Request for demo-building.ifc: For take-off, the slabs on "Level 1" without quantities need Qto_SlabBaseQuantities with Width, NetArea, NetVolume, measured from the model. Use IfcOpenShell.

First a look at what the model holds.

```python
import ifcopenshell
import ifcopenshell.util.element
import ifcopenshell.util.unit

model = ifcopenshell.open("demo-building.ifc")
print(model.schema)
for unit_type in ("LENGTHUNIT", "AREAUNIT", "VOLUMEUNIT"):
    print(unit_type, ifcopenshell.util.unit.calculate_unit_scale(model, unit_type))
storey = next(s for s in model.by_type("IfcBuildingStorey") if s.Name == "Level 1")
slabs = [e for e in ifcopenshell.util.element.get_decomposition(storey) if e.is_a("IfcSlab")]
for e in sorted(slabs, key=lambda e: e.id()):
    print(e.id(), e.is_a(), e.Name, list(ifcopenshell.util.element.get_psets(e, qtos_only=True)), sep=" | ")
```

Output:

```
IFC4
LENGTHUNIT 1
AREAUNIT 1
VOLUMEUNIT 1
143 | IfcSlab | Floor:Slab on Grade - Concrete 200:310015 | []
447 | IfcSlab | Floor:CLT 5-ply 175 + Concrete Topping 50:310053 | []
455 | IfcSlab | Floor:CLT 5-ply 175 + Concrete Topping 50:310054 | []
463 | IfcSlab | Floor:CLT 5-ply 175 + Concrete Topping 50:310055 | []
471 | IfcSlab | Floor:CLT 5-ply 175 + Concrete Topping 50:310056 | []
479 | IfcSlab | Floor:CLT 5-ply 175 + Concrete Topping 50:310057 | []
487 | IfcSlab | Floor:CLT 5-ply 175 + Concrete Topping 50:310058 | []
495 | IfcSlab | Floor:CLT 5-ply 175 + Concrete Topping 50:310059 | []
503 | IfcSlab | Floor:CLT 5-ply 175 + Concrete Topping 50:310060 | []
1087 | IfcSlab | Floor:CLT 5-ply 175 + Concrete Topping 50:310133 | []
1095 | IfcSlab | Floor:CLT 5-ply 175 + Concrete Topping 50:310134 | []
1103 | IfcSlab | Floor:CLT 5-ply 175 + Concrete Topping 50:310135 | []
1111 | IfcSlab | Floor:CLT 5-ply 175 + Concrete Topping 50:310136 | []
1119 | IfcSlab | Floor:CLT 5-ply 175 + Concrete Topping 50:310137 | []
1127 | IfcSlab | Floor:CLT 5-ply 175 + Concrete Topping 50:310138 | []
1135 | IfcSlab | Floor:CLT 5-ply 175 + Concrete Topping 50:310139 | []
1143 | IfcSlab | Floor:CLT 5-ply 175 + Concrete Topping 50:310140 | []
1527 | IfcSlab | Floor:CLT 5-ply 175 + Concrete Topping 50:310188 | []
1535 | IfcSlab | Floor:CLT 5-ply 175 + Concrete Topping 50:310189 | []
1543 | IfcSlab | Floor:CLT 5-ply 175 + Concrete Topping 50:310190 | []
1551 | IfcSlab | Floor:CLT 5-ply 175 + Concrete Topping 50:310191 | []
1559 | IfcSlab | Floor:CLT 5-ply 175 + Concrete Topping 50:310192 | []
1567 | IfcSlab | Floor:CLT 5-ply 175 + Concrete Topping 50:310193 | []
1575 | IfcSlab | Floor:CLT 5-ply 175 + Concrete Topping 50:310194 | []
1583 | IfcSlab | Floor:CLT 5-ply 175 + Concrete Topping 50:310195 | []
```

```python
import ifcopenshell
import ifcopenshell.api.pset
import ifcopenshell.geom
import ifcopenshell.util.element
import ifcopenshell.util.shape
import ifcopenshell.util.unit

model = ifcopenshell.open("demo-building.ifc")
unit_scale = ifcopenshell.util.unit.calculate_unit_scale(model)
area_scale = ifcopenshell.util.unit.calculate_unit_scale(model, "AREAUNIT")
volume_scale = ifcopenshell.util.unit.calculate_unit_scale(model, "VOLUMEUNIT")
settings = ifcopenshell.geom.settings()

storey = next(s for s in model.by_type("IfcBuildingStorey") if s.Name == "Level 1")
slabs = [e for e in ifcopenshell.util.element.get_decomposition(storey) if e.is_a("IfcSlab")]

for e in sorted(slabs, key=lambda e: e.id()):
    if ifcopenshell.util.element.get_psets(e, qtos_only=True, should_inherit=False):
        continue
    # Geometry comes back in metres, in the element's own axes.
    shape = ifcopenshell.geom.create_shape(settings, e)
    values = {
        "Width": ifcopenshell.util.shape.get_z(shape.geometry) / unit_scale,
        "NetArea": ifcopenshell.util.shape.get_footprint_area(shape.geometry) / area_scale,
        "NetVolume": ifcopenshell.util.shape.get_volume(shape.geometry) / volume_scale,
    }
    qto = ifcopenshell.api.pset.add_qto(model, product=e, name="Qto_SlabBaseQuantities")
    ifcopenshell.api.pset.edit_qto(model, qto=qto, properties=values)
    print(e.id(), {k: round(v, 3) for k, v in values.items()})

model.write("demo-building_updated.ifc")
```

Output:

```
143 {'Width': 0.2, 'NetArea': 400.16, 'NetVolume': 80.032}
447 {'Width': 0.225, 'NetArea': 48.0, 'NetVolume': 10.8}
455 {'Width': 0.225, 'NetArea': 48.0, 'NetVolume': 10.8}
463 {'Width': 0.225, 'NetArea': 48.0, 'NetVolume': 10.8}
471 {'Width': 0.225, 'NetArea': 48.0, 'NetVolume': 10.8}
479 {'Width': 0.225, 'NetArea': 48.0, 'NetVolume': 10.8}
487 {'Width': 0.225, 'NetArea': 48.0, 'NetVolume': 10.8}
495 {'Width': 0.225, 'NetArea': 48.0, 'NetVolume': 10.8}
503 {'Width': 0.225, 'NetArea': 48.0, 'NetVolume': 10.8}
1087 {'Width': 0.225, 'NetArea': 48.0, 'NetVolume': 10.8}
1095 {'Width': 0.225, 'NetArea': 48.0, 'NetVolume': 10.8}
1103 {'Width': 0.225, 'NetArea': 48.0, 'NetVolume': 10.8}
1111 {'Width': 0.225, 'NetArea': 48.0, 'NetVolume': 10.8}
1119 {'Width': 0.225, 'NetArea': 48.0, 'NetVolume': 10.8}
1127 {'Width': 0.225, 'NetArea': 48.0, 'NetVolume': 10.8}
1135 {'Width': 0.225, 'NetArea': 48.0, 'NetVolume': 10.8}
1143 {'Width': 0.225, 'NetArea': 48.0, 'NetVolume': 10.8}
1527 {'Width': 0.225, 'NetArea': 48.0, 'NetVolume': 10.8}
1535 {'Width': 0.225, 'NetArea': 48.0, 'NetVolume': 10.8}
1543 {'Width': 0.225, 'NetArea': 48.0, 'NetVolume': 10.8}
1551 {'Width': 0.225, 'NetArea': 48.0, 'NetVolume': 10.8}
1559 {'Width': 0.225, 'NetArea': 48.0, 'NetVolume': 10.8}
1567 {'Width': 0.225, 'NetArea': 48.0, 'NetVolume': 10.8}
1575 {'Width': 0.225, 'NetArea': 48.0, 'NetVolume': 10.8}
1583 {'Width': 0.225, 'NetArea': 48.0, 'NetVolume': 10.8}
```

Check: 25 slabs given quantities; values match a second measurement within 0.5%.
